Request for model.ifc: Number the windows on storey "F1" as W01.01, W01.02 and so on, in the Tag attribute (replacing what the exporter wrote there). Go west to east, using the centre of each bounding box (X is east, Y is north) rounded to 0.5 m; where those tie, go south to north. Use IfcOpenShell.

First a look at what the model holds.

```python
import ifcopenshell
import ifcopenshell.util.element
import ifcopenshell.util.placement

model = ifcopenshell.open("model.ifc")
print(model.schema)
storey = next(s for s in model.by_type("IfcBuildingStorey") if s.Name == "F1")
windows = [e for e in ifcopenshell.util.element.get_decomposition(storey) if e.is_a("IfcWindow")]
for e in sorted(windows, key=lambda e: e.id()):
    origin = ifcopenshell.util.placement.get_local_placement(e.ObjectPlacement)[:3, 3]
    print(e.id(), e.Tag, e.Name, origin.round(2) + 0.0, sep=" | ")
```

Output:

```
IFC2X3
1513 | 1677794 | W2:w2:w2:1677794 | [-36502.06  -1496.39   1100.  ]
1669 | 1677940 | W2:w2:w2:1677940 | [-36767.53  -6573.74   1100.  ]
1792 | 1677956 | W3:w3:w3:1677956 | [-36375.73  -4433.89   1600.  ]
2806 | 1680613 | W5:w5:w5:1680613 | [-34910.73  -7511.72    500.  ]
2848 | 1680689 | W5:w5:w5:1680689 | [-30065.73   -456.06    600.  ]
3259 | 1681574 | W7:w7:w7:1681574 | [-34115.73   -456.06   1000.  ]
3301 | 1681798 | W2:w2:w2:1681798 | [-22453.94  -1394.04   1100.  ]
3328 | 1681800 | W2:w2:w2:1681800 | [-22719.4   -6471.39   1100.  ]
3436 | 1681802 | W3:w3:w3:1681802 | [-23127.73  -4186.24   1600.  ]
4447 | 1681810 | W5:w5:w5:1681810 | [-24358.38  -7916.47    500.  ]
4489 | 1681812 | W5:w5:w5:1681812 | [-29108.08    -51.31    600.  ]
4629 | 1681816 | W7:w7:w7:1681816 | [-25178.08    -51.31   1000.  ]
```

```python
import ifcopenshell
import ifcopenshell.geom
import ifcopenshell.util.element
import ifcopenshell.util.shape

model = ifcopenshell.open("model.ifc")
settings = ifcopenshell.geom.settings()
settings.set("use-world-coords", True)


def centre(element):
    shape = ifcopenshell.geom.create_shape(settings, element)
    return ifcopenshell.util.shape.get_bbox_centroid(shape.geometry)


storey = next(s for s in model.by_type("IfcBuildingStorey") if s.Name == "F1")
windows = [e for e in ifcopenshell.util.element.get_decomposition(storey) if e.is_a("IfcWindow")]

# Insertion points can sit at a corner or the storey origin, so sort by the geometry (in metres).
centres = {e: centre(e) for e in windows}
windows.sort(key=lambda e: (round(centres[e][0] / 0.5), centres[e][1]))

for i, e in enumerate(windows, start=1):
    number = f"W01.{i:02d}"
    e.Tag = number
    print(e.id(), number)

model.write("model_v2.ifc")
```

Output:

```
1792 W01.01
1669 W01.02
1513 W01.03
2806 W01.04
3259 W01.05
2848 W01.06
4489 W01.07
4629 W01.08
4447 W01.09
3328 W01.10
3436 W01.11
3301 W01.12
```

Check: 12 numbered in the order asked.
